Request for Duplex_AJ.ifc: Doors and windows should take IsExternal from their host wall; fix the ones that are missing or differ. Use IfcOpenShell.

First a look at what the model holds.

```python
import ifcopenshell
import ifcopenshell.util.element

model = ifcopenshell.open("Duplex_AJ.ifc")
print(model.schema)
seen = {}
for e in model.by_type("IfcDoor") + model.by_type("IfcWindow"):
    if not e.FillsVoids:
        continue
    host = e.FillsVoids[0].RelatingOpeningElement.VoidsElements[0].RelatingBuildingElement
    own = ifcopenshell.util.element.get_pset(e, f"Pset_{e.is_a()[3:].removesuffix('StandardCase')}Common", "IsExternal")
    wall = ifcopenshell.util.element.get_pset(host, "Pset_WallCommon", "IsExternal")
    seen[e.is_a(), own, wall] = seen.get((e.is_a(), own, wall), 0) + 1
for (cls, own, wall), count in sorted(seen.items(), key=str):
    print(count, cls, "IsExternal:", own, "| host wall:", wall)
```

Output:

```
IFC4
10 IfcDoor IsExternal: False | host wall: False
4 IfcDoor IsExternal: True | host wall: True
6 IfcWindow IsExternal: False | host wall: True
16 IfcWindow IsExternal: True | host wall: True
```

```python
import ifcopenshell
import ifcopenshell.api.pset
import ifcopenshell.util.element

model = ifcopenshell.open("Duplex_AJ.ifc")

count = 0
for ifc_class, pset_name in (("IfcDoor", "Pset_DoorCommon"), ("IfcWindow", "Pset_WindowCommon")):
    for e in model.by_type(ifc_class):
        if not e.FillsVoids:
            continue
        host = e.FillsVoids[0].RelatingOpeningElement.VoidsElements[0].RelatingBuildingElement
        external = ifcopenshell.util.element.get_pset(host, "Pset_WallCommon", "IsExternal")
        if external is None or ifcopenshell.util.element.get_pset(e, pset_name, "IsExternal") == external:
            continue
        pset = ifcopenshell.api.pset.add_pset(model, product=e, name=pset_name)
        ifcopenshell.api.pset.edit_pset(model, pset=pset, properties={"IsExternal": external})
        count += 1

print(count, "updated")

model.write("Duplex_AJ_edited.ifc")
```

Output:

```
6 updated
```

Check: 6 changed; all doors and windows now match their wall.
